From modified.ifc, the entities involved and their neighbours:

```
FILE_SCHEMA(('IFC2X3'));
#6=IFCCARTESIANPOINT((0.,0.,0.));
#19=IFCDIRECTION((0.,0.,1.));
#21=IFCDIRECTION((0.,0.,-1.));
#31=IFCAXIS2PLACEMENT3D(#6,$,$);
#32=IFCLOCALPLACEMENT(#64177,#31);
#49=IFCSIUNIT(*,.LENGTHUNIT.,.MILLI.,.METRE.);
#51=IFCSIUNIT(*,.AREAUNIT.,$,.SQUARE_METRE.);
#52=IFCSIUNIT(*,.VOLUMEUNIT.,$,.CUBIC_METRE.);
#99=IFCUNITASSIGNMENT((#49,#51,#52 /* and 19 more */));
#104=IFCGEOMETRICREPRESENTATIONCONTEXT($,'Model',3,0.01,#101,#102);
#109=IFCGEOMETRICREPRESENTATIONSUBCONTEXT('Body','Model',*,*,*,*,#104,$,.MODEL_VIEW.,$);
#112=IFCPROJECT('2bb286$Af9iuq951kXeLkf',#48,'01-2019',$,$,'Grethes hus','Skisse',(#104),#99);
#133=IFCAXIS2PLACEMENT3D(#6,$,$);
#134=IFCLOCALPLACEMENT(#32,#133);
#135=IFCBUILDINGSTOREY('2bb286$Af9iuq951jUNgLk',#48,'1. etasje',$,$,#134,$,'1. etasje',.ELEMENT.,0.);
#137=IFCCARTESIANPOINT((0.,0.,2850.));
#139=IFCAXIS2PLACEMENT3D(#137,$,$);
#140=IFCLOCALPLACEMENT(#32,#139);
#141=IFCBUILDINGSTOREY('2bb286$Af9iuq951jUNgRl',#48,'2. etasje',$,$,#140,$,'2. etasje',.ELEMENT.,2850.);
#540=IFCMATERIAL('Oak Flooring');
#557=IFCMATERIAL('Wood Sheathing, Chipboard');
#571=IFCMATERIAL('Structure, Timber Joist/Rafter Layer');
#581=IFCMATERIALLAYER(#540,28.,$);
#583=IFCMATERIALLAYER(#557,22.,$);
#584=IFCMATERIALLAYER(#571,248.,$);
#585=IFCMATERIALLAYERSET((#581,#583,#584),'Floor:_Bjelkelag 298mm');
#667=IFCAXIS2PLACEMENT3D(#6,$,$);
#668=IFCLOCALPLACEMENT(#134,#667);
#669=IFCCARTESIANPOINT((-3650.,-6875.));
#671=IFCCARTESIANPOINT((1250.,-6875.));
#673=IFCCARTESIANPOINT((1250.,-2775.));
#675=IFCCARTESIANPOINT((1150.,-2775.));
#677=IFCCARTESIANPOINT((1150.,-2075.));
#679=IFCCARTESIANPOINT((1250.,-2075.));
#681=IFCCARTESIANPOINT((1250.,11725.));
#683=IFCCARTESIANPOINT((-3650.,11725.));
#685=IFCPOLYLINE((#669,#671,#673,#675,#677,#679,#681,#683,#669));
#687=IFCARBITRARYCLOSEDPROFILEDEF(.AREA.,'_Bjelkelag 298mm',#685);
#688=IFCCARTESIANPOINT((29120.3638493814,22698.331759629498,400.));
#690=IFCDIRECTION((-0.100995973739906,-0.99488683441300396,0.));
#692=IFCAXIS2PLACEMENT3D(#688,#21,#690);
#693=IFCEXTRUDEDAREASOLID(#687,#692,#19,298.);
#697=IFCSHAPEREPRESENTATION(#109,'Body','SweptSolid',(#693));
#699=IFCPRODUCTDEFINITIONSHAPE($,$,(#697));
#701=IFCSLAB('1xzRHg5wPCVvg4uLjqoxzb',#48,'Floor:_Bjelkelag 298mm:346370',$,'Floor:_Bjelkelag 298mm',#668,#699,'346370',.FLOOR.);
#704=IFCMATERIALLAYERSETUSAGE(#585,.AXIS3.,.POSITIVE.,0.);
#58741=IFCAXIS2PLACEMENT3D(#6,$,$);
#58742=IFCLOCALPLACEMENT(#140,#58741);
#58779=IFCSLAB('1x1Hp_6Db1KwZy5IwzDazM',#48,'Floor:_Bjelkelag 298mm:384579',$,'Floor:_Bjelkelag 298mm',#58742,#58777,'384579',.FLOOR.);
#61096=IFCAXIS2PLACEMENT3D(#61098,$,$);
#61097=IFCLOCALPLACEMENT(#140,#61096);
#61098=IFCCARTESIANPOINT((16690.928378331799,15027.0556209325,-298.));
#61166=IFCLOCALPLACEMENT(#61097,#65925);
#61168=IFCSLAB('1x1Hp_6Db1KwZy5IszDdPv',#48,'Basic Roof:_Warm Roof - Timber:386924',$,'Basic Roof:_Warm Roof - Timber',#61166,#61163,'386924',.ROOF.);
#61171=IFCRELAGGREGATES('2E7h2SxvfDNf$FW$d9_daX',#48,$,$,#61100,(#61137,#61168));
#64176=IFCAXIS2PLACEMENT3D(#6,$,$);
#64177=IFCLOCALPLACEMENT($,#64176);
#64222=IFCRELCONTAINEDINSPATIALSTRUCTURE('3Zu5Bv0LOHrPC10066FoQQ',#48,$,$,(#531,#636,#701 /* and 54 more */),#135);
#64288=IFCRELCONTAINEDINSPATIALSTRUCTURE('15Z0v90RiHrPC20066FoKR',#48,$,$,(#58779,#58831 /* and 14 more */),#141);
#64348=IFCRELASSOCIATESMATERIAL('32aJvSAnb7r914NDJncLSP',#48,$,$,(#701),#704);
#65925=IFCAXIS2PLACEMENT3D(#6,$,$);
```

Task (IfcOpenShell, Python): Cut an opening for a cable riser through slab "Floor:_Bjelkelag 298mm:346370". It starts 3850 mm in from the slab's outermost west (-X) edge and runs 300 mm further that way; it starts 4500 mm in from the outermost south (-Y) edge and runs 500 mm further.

```python
import numpy as np
import ifcopenshell
import ifcopenshell.api.feature
import ifcopenshell.api.geometry
import ifcopenshell.api.root
import ifcopenshell.geom
import ifcopenshell.util.placement
import ifcopenshell.util.representation
import ifcopenshell.util.shape
import ifcopenshell.util.unit

model = ifcopenshell.open("modified.ifc")
unit_scale = ifcopenshell.util.unit.calculate_unit_scale(model)
settings = ifcopenshell.geom.settings()


def volume(element):
    """Net volume in cubic metres, openings subtracted."""
    shape = ifcopenshell.geom.create_shape(settings, element)
    return ifcopenshell.util.shape.get_volume(shape.geometry)


slab = model.by_guid("1xzRHg5wPCVvg4uLjqoxzb")
before = volume(slab)

# Extent in the slab's own axes, in metres. The edges named are its -X and -Y sides.
slab_shape = ifcopenshell.geom.create_shape(settings, slab)
vertices = ifcopenshell.util.shape.get_vertices(slab_shape.geometry)
x_min, y_min, bottom = vertices.min(axis=0)
top = vertices[:, 2].max()

opening = ifcopenshell.api.root.create_entity(model, ifc_class="IfcOpeningElement", name="Cable riser opening")
context = ifcopenshell.util.representation.get_context(model, "Model", "Body", "MODEL_VIEW")
width, depth = 0.3, 0.5
outline = [(0.0, 0.0), (width, 0.0), (width, depth), (0.0, depth), (0.0, 0.0)]
# Overshoot both faces by 50 mm so the cut is clean.
shape = ifcopenshell.api.geometry.add_slab_representation(
    model, context=context, depth=top - bottom + 0.1, polyline=outline
)
ifcopenshell.api.geometry.assign_representation(model, product=opening, representation=shape)

matrix = ifcopenshell.util.placement.get_local_placement(slab.ObjectPlacement)
matrix[:, 3] = matrix @ np.append(np.array([x_min + 3.85, y_min + 4.5, bottom - 0.05]) / unit_scale, 1.0)
ifcopenshell.api.geometry.edit_object_placement(model, product=opening, matrix=matrix, is_si=False)
ifcopenshell.api.feature.add_feature(model, feature=opening, element=slab)

after = volume(slab)

print(f"slab volume {before:.3f} -> {after:.3f} m3")

model.write("modified_updated.ifc")
```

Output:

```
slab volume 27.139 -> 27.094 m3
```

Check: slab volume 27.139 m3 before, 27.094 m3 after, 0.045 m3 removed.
